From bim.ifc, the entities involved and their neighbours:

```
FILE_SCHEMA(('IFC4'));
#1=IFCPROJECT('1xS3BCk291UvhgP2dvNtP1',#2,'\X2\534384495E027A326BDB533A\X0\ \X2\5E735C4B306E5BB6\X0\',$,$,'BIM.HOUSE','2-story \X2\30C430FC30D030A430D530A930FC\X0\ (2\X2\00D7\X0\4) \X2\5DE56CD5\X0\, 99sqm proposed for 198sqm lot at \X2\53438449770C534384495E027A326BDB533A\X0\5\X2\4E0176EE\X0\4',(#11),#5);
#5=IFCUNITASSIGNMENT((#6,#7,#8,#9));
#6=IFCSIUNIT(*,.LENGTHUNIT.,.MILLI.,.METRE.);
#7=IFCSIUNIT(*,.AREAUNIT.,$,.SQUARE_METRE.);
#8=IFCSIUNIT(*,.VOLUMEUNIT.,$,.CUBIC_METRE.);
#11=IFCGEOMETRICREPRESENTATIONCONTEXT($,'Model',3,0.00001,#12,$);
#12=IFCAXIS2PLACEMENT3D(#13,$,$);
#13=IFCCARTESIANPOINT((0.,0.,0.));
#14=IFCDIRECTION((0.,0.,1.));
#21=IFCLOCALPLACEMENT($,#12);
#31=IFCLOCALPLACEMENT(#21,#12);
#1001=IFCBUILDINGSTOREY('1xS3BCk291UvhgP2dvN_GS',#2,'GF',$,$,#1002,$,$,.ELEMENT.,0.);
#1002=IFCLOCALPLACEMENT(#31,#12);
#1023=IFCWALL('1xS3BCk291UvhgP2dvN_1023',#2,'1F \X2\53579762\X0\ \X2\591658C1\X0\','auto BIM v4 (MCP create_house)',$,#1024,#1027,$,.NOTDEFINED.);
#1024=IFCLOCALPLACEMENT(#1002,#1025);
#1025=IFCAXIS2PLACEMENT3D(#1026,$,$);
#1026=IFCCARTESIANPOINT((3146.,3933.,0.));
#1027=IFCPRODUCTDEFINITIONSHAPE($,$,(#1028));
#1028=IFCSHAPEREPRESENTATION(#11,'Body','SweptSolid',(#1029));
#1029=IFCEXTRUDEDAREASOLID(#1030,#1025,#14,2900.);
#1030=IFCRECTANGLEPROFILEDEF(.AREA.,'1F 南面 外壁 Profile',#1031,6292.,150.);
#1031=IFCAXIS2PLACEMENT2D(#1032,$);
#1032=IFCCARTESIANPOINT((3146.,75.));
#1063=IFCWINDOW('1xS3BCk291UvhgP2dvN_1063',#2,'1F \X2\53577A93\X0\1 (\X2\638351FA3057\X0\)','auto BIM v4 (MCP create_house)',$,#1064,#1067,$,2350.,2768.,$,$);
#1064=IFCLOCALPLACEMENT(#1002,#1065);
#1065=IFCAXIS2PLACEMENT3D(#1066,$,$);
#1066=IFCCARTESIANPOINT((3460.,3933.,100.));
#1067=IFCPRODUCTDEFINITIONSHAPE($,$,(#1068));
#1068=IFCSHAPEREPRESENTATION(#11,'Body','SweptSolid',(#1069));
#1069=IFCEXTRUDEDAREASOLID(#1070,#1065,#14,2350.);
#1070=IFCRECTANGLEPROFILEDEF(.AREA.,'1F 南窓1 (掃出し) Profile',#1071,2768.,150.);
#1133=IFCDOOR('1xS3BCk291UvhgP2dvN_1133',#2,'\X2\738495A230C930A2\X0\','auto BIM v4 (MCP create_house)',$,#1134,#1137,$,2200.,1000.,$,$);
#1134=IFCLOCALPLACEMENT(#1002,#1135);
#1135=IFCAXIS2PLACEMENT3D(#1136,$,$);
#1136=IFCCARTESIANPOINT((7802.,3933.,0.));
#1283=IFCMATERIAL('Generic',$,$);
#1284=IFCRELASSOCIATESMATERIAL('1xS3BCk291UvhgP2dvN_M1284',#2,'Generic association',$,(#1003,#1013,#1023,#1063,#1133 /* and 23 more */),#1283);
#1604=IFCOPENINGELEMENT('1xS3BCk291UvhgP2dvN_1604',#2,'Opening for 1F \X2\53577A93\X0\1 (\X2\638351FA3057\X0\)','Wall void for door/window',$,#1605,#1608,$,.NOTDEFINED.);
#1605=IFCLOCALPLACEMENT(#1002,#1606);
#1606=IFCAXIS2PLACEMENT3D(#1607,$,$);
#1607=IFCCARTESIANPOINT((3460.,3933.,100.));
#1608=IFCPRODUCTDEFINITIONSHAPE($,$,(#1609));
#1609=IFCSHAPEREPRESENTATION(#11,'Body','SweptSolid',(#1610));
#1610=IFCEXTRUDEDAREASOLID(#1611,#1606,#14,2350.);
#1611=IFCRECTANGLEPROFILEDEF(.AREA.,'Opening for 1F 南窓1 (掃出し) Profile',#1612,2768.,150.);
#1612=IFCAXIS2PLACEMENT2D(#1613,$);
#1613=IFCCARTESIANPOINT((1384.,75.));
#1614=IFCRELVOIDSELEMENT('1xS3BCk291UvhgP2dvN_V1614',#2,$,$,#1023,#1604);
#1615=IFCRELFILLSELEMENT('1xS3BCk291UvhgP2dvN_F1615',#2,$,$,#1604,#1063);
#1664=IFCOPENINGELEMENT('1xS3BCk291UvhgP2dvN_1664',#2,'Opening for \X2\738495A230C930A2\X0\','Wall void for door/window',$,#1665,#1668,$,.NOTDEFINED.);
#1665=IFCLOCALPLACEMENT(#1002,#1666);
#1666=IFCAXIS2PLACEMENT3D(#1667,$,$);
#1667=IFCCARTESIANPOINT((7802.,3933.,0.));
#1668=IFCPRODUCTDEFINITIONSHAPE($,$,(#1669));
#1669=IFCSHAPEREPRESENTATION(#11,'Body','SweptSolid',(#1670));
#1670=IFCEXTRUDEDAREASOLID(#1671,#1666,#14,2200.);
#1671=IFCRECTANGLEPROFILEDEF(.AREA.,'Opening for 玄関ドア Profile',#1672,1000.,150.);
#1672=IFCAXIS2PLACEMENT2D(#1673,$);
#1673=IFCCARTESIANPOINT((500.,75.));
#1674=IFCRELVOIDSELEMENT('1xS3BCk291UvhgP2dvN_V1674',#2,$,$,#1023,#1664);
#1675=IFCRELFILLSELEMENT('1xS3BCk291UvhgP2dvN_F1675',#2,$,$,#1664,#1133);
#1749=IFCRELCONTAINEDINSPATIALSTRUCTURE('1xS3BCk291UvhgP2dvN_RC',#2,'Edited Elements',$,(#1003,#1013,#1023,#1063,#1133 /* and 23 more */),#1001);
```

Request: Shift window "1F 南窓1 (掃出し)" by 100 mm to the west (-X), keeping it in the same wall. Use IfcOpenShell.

```python
import ifcopenshell
import ifcopenshell.api.geometry
import ifcopenshell.util.placement
import ifcopenshell.util.unit

model = ifcopenshell.open("bim.ifc")
unit_scale = ifcopenshell.util.unit.calculate_unit_scale(model)

window = model.by_guid("1xS3BCk291UvhgP2dvN_1063")
opening = window.FillsVoids[0].RelatingOpeningElement
wall = opening.VoidsElements[0].RelatingBuildingElement

wall_matrix = ifcopenshell.util.placement.get_local_placement(wall.ObjectPlacement)
shift = wall_matrix[:3, 0] * -0.1 / unit_scale
before = ifcopenshell.util.placement.get_local_placement(window.ObjectPlacement)[:3, 3].copy()

# The window is not placed relative to its opening, so move both.
for product in (opening, window):
    matrix = ifcopenshell.util.placement.get_local_placement(product.ObjectPlacement)
    matrix[:3, 3] += shift
    ifcopenshell.api.geometry.edit_object_placement(model, product=product, matrix=matrix, is_si=False)

after = ifcopenshell.util.placement.get_local_placement(window.ObjectPlacement)[:3, 3]
print("window moved by", (after - before).round(3) + 0.0)

model.write("bim_rev.ifc")
```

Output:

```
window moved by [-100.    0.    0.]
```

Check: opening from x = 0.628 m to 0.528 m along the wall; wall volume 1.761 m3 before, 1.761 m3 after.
